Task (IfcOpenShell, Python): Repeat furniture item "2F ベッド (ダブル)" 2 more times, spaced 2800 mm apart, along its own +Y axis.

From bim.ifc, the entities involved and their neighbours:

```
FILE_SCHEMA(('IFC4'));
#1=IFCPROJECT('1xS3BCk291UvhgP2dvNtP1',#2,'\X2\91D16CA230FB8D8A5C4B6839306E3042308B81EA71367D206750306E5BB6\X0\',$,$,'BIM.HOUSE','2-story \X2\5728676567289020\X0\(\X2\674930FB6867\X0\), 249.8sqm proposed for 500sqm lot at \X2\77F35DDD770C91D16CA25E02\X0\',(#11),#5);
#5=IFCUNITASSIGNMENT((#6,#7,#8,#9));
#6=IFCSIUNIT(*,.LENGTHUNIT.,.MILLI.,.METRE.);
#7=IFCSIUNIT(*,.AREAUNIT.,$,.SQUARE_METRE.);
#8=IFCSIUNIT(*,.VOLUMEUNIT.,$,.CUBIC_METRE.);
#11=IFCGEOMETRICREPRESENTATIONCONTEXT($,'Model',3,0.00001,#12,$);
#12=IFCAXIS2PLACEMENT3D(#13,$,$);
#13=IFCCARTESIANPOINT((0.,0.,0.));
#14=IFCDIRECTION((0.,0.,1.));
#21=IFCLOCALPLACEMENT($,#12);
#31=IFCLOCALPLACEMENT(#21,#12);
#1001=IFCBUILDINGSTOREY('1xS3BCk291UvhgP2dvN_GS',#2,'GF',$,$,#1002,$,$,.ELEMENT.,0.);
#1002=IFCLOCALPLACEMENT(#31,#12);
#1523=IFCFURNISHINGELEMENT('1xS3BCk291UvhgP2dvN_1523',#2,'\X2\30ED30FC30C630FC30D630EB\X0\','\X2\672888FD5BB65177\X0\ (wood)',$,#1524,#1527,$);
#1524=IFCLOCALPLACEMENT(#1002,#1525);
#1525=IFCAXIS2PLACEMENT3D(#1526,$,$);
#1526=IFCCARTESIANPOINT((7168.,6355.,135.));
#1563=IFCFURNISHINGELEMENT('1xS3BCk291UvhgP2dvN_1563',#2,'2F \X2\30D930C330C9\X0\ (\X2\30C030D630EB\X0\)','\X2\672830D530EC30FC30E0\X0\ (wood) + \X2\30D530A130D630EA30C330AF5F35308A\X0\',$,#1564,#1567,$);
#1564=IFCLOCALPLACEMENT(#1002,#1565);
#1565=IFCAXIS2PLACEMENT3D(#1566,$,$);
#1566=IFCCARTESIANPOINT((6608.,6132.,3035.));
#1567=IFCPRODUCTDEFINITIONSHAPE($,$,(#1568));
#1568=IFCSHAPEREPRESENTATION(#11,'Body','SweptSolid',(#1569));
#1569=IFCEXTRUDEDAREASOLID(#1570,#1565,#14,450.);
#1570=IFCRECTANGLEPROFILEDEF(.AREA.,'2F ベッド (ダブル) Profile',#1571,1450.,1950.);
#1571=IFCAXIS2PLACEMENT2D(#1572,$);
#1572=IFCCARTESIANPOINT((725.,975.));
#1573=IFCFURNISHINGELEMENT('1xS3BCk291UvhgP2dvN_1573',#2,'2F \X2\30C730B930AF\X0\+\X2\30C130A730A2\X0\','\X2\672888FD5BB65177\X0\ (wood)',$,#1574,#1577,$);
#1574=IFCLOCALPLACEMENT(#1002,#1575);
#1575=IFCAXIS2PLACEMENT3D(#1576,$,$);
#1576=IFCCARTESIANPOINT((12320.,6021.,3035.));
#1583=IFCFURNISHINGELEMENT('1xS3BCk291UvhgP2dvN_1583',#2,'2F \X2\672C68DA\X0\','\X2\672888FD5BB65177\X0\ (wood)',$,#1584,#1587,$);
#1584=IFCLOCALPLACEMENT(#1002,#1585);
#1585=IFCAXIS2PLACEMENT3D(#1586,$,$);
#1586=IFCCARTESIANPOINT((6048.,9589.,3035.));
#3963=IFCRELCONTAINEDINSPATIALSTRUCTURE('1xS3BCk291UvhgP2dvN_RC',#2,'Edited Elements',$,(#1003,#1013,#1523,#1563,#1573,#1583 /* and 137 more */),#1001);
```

```python
import ifcopenshell
import ifcopenshell.api.geometry
import ifcopenshell.api.root
import ifcopenshell.util.element
import ifcopenshell.util.placement
import ifcopenshell.util.unit

model = ifcopenshell.open("bim.ifc")
unit_scale = ifcopenshell.util.unit.calculate_unit_scale(model)


def reuse_history(source, copy):
    """copy_class also copies each property set's owner history, people and application; keep the originals."""
    for rel in copy.IsDefinedBy:
        if rel.is_a("IfcRelDefinesByProperties") and (history := rel.RelatingPropertyDefinition.OwnerHistory):
            rel.RelatingPropertyDefinition.OwnerHistory = source.OwnerHistory
            ifcopenshell.util.element.remove_deep2(model, history)


source = model.by_guid("1xS3BCk291UvhgP2dvN_1563")
base = ifcopenshell.util.placement.get_local_placement(source.ObjectPlacement)
step = base[:3, 1] * 2.8 / unit_scale

for i in range(1, 3):
    copy = ifcopenshell.api.root.copy_class(model, product=source)
    copy.Representation = ifcopenshell.util.element.copy_deep(
        model, source.Representation, exclude=["IfcGeometricRepresentationContext", "IfcRepresentationMap"]
    )
    reuse_history(source, copy)
    matrix = base.copy()
    matrix[:3, 3] += i * step
    print("added at", matrix[:3, 3].round(3) + 0.0)
    ifcopenshell.api.geometry.edit_object_placement(model, product=copy, matrix=matrix, is_si=False)

model.write("bim_rev.ifc")
```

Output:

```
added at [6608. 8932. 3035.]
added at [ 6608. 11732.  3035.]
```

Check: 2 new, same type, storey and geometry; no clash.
